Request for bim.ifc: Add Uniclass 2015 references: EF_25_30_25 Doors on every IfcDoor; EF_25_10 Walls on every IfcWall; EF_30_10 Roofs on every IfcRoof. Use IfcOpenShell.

First a look at what the model holds.

```python
import ifcopenshell

model = ifcopenshell.open("bim.ifc")
print(model.schema)
print("classifications:", [c.Name for c in model.by_type("IfcClassification")])
for ifc_class in ("IfcDoor", "IfcRoof", "IfcStair", "IfcWall", "IfcWindow"):
    print(ifc_class, len(model.by_type(ifc_class)))
```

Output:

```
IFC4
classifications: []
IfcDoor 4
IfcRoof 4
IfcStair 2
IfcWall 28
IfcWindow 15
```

```python
import ifcopenshell
import ifcopenshell.api.classification

model = ifcopenshell.open("bim.ifc")

system = ifcopenshell.api.classification.add_classification(model, classification="Uniclass 2015")

codes = {
    "IfcDoor": ("EF_25_30_25", "Doors"),
    "IfcWall": ("EF_25_10", "Walls"),
    "IfcRoof": ("EF_30_10", "Roofs"),
}
for ifc_class, (code, name) in codes.items():
    products = model.by_type(ifc_class)
    ifcopenshell.api.classification.add_reference(
        model, products=products, classification=system, identification=code, name=name
    )
    print(code, len(products))

model.write("bim_edited.ifc")
```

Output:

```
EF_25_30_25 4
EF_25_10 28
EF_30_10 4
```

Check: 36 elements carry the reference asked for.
